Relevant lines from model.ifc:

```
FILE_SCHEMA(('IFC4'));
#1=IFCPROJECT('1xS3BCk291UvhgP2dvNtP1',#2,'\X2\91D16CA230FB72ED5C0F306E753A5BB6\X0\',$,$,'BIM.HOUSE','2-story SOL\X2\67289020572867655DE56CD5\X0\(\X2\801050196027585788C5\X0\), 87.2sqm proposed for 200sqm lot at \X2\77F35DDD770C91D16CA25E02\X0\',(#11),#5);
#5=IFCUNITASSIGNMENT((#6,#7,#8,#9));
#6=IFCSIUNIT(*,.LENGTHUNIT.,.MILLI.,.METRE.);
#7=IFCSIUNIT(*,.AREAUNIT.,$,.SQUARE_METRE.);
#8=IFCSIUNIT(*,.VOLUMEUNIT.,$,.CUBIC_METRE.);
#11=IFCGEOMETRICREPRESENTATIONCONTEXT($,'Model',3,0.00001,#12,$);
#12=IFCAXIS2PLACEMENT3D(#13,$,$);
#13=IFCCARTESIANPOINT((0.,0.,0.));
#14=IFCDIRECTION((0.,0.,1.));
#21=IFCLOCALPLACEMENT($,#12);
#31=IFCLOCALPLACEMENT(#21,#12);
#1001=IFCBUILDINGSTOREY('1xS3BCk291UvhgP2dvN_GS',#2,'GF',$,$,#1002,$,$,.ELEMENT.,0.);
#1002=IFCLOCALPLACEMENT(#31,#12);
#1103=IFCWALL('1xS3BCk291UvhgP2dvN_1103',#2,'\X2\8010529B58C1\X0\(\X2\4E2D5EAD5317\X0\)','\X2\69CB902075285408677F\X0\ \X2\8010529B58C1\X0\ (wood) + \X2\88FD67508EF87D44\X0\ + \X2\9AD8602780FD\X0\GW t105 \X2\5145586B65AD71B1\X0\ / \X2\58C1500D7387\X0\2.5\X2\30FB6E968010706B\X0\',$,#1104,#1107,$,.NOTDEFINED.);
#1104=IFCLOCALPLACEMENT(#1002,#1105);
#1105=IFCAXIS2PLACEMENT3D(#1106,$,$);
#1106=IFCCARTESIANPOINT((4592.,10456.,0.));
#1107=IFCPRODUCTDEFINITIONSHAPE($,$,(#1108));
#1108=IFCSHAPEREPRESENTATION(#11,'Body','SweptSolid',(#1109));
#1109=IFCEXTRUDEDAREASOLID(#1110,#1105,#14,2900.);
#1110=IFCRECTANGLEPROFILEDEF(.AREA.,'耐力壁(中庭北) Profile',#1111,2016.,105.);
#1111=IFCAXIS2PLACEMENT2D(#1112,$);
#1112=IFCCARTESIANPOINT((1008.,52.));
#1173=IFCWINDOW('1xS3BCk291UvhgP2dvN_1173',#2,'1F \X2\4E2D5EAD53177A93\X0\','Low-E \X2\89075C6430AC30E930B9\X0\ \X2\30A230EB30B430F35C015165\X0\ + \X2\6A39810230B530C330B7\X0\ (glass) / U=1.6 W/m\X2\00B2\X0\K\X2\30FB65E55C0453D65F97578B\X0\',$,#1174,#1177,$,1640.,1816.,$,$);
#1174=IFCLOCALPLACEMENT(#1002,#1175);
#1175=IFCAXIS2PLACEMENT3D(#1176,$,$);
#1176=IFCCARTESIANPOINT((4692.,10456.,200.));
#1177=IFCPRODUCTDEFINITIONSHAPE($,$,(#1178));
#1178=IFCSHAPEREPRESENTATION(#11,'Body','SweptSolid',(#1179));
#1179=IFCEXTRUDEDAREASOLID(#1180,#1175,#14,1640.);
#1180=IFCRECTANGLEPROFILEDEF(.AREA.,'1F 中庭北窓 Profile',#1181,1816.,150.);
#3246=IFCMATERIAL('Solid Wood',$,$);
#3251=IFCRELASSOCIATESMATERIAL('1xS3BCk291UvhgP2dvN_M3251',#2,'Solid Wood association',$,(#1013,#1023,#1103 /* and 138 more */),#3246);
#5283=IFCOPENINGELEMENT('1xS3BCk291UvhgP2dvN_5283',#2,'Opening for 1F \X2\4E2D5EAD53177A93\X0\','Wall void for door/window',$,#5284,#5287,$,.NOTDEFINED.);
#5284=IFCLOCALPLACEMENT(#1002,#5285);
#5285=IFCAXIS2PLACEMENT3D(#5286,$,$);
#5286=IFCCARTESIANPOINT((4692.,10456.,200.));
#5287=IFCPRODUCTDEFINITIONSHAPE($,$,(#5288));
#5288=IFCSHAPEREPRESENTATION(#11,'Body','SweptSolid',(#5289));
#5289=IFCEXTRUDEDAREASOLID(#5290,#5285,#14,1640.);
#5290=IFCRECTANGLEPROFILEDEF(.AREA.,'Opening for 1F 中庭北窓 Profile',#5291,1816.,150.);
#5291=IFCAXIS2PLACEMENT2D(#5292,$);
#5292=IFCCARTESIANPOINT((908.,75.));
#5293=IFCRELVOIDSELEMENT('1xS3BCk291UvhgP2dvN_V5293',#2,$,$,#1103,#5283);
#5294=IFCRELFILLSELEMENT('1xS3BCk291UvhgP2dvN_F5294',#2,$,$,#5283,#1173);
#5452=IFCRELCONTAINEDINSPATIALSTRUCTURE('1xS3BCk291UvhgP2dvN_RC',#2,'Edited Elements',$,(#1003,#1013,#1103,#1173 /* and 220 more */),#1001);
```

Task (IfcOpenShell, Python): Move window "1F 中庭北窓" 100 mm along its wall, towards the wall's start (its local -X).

```python
import ifcopenshell
import ifcopenshell.api.geometry
import ifcopenshell.util.placement

model = ifcopenshell.open("model.ifc")

window = model.by_guid("1xS3BCk291UvhgP2dvN_1173")
opening = window.FillsVoids[0].RelatingOpeningElement
wall = opening.VoidsElements[0].RelatingBuildingElement

wall_matrix = ifcopenshell.util.placement.get_local_placement(wall.ObjectPlacement)
shift = wall_matrix[:3, 0] * -100.0
before = ifcopenshell.util.placement.get_local_placement(window.ObjectPlacement)[:3, 3].copy()

# The window is not placed relative to its opening, so move both.
for product in (opening, window):
    matrix = ifcopenshell.util.placement.get_local_placement(product.ObjectPlacement)
    matrix[:3, 3] += shift
    ifcopenshell.api.geometry.edit_object_placement(model, product=product, matrix=matrix, is_si=False)

after = ifcopenshell.util.placement.get_local_placement(window.ObjectPlacement)[:3, 3]
print("window moved by", (after - before).round(3) + 0.0)

model.write("model-out.ifc")
```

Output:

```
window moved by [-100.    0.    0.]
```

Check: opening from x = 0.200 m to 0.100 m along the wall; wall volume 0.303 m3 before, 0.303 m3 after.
